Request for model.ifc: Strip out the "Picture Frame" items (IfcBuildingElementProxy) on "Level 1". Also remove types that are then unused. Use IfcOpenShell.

First a look at what the model holds.

```python
import ifcopenshell
import ifcopenshell.util.element

model = ifcopenshell.open("model.ifc")
print(model.schema)
storey = next(s for s in model.by_type("IfcBuildingStorey") if s.Name == "Level 1")
proxies = [e for e in ifcopenshell.util.element.get_decomposition(storey) if e.is_a("IfcBuildingElementProxy")]
seen = {}
for e in proxies:
    element_type = ifcopenshell.util.element.get_type(e)
    name = element_type.Name if element_type not in (None, e) else None
    seen[name] = seen.get(name, 0) + 1
for name, count in sorted(seen.items(), key=str):
    print(count, "x", name)
```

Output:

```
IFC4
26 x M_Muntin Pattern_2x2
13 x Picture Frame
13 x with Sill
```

```python
import ifcopenshell
import ifcopenshell.api.root
import ifcopenshell.util.element

model = ifcopenshell.open("model.ifc")

storey = next(s for s in model.by_type("IfcBuildingStorey") if s.Name == "Level 1")
proxies = [e for e in ifcopenshell.util.element.get_decomposition(storey) if e.is_a("IfcBuildingElementProxy")]
targets = [e for e in proxies if (t := ifcopenshell.util.element.get_type(e)) not in (None, e) and t.Name == "Picture Frame"]
types = {ifcopenshell.util.element.get_type(e) for e in targets} - {None, *targets}

for e in targets:
    ifcopenshell.api.root.remove_product(model, product=e)
print(len(targets), "removed")

unused = [t for t in types if not ifcopenshell.util.element.get_types(t)]
for t in unused:
    ifcopenshell.api.root.remove_product(model, product=t)
print(len(unused), "unused types removed")

model.write("model_v2.ifc")
```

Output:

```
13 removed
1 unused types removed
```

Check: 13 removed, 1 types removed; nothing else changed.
